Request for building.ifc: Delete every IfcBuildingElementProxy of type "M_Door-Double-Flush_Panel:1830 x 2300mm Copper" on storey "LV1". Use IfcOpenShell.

First a look at what the model holds.

```python
import ifcopenshell
import ifcopenshell.util.element

model = ifcopenshell.open("building.ifc")
print(model.schema)
storey = next(s for s in model.by_type("IfcBuildingStorey") if s.Name == "LV1")
proxies = [e for e in ifcopenshell.util.element.get_decomposition(storey) if e.is_a("IfcBuildingElementProxy")]
seen = {}
for e in proxies:
    element_type = ifcopenshell.util.element.get_type(e)
    name = element_type.Name if element_type not in (None, e) else None
    seen[name] = seen.get(name, 0) + 1
for name, count in sorted(seen.items(), key=str):
    print(count, "x", name)
```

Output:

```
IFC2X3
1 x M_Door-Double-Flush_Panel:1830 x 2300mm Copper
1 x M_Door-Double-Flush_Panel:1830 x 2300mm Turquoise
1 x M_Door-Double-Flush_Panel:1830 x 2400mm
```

```python
import ifcopenshell
import ifcopenshell.api.root
import ifcopenshell.util.element

model = ifcopenshell.open("building.ifc")

storey = next(s for s in model.by_type("IfcBuildingStorey") if s.Name == "LV1")
proxies = [e for e in ifcopenshell.util.element.get_decomposition(storey) if e.is_a("IfcBuildingElementProxy")]
targets = [e for e in proxies if (t := ifcopenshell.util.element.get_type(e)) not in (None, e) and t.Name == "M_Door-Double-Flush_Panel:1830 x 2300mm Copper"]

for e in targets:
    ifcopenshell.api.root.remove_product(model, product=e)
print(len(targets), "removed")

model.write("building_v2.ifc")
```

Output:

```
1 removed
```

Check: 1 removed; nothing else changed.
